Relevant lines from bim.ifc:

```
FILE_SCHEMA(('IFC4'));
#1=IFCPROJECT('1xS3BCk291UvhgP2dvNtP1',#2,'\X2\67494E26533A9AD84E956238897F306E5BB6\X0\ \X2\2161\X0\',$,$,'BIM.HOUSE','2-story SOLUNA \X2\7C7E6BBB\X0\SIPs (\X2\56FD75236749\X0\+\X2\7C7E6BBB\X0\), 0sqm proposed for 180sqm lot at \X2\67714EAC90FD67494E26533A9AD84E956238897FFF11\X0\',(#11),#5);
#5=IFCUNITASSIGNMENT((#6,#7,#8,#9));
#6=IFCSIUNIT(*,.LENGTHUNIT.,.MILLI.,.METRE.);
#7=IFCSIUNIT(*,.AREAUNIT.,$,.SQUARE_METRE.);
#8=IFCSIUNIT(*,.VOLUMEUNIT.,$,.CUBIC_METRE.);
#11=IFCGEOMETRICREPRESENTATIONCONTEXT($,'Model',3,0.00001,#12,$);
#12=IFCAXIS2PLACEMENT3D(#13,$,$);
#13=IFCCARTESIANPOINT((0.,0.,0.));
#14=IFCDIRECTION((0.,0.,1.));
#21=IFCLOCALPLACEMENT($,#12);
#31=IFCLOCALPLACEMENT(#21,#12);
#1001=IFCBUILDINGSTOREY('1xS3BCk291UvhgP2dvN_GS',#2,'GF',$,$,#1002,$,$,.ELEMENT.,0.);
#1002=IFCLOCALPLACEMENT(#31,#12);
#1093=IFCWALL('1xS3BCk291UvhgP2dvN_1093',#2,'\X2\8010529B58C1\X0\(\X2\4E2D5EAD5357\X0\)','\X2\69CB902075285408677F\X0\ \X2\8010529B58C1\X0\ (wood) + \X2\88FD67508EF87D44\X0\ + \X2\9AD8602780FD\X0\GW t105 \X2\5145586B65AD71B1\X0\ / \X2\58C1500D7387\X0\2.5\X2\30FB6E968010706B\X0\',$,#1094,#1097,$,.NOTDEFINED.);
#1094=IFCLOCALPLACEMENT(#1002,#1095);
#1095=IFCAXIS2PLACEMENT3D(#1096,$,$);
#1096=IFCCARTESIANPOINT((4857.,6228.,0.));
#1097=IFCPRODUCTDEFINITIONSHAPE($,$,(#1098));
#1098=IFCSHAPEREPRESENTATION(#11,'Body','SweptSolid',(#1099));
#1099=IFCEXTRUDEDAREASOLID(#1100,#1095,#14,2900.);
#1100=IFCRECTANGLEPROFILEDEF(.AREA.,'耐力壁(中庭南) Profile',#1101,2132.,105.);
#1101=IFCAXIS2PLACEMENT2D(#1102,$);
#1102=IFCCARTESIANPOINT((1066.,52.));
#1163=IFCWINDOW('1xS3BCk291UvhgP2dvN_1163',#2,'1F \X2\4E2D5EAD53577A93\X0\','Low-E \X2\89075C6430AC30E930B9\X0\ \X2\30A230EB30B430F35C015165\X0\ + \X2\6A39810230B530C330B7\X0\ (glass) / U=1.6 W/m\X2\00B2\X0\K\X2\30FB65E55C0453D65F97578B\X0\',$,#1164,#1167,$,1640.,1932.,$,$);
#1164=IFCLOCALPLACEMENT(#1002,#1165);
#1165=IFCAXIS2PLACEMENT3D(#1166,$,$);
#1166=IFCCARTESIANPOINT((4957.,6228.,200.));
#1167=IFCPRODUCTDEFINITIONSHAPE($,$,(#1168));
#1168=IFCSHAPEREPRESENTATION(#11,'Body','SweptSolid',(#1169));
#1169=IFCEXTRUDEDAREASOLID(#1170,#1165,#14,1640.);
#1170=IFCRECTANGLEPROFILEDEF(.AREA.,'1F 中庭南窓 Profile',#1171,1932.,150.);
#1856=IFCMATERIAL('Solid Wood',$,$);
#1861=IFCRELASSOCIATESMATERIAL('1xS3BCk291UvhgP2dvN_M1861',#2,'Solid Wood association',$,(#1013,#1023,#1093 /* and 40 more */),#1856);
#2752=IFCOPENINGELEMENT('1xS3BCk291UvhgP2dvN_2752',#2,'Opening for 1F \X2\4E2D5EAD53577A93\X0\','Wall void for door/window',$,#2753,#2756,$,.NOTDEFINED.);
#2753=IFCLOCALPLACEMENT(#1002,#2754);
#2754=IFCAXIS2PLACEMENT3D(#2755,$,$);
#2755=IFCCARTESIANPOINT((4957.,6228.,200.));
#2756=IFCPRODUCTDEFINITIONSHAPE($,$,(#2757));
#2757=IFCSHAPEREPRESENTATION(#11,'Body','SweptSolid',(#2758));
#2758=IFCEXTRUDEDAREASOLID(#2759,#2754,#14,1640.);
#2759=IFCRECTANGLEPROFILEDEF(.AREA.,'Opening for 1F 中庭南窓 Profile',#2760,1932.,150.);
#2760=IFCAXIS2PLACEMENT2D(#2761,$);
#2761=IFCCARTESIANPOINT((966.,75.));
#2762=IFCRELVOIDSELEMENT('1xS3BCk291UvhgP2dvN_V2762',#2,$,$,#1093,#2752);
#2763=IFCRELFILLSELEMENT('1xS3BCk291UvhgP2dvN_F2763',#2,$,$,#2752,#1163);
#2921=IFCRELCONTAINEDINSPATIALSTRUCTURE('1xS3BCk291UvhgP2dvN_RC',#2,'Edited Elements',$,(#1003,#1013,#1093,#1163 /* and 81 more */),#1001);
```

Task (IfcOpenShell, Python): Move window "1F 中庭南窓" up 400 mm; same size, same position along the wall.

```python
import numpy as np
import ifcopenshell
import ifcopenshell.api.geometry
import ifcopenshell.util.placement
import ifcopenshell.util.unit

model = ifcopenshell.open("bim.ifc")
unit_scale = ifcopenshell.util.unit.calculate_unit_scale(model)

window = model.by_guid("1xS3BCk291UvhgP2dvN_1163")
opening = window.FillsVoids[0].RelatingOpeningElement
dz = 0.4 / unit_scale

shift = np.array([0.0, 0.0, dz])
# The window is not placed relative to its opening, so move both.
for product in (opening, window):
    matrix = ifcopenshell.util.placement.get_local_placement(product.ObjectPlacement)
    matrix[:3, 3] += shift
    ifcopenshell.api.geometry.edit_object_placement(model, product=product, matrix=matrix, is_si=False)

print(f"moved by {dz * unit_scale:+.3f} m")

model.write("bim_edited.ifc")
```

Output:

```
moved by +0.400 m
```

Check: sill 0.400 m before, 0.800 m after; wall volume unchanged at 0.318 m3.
